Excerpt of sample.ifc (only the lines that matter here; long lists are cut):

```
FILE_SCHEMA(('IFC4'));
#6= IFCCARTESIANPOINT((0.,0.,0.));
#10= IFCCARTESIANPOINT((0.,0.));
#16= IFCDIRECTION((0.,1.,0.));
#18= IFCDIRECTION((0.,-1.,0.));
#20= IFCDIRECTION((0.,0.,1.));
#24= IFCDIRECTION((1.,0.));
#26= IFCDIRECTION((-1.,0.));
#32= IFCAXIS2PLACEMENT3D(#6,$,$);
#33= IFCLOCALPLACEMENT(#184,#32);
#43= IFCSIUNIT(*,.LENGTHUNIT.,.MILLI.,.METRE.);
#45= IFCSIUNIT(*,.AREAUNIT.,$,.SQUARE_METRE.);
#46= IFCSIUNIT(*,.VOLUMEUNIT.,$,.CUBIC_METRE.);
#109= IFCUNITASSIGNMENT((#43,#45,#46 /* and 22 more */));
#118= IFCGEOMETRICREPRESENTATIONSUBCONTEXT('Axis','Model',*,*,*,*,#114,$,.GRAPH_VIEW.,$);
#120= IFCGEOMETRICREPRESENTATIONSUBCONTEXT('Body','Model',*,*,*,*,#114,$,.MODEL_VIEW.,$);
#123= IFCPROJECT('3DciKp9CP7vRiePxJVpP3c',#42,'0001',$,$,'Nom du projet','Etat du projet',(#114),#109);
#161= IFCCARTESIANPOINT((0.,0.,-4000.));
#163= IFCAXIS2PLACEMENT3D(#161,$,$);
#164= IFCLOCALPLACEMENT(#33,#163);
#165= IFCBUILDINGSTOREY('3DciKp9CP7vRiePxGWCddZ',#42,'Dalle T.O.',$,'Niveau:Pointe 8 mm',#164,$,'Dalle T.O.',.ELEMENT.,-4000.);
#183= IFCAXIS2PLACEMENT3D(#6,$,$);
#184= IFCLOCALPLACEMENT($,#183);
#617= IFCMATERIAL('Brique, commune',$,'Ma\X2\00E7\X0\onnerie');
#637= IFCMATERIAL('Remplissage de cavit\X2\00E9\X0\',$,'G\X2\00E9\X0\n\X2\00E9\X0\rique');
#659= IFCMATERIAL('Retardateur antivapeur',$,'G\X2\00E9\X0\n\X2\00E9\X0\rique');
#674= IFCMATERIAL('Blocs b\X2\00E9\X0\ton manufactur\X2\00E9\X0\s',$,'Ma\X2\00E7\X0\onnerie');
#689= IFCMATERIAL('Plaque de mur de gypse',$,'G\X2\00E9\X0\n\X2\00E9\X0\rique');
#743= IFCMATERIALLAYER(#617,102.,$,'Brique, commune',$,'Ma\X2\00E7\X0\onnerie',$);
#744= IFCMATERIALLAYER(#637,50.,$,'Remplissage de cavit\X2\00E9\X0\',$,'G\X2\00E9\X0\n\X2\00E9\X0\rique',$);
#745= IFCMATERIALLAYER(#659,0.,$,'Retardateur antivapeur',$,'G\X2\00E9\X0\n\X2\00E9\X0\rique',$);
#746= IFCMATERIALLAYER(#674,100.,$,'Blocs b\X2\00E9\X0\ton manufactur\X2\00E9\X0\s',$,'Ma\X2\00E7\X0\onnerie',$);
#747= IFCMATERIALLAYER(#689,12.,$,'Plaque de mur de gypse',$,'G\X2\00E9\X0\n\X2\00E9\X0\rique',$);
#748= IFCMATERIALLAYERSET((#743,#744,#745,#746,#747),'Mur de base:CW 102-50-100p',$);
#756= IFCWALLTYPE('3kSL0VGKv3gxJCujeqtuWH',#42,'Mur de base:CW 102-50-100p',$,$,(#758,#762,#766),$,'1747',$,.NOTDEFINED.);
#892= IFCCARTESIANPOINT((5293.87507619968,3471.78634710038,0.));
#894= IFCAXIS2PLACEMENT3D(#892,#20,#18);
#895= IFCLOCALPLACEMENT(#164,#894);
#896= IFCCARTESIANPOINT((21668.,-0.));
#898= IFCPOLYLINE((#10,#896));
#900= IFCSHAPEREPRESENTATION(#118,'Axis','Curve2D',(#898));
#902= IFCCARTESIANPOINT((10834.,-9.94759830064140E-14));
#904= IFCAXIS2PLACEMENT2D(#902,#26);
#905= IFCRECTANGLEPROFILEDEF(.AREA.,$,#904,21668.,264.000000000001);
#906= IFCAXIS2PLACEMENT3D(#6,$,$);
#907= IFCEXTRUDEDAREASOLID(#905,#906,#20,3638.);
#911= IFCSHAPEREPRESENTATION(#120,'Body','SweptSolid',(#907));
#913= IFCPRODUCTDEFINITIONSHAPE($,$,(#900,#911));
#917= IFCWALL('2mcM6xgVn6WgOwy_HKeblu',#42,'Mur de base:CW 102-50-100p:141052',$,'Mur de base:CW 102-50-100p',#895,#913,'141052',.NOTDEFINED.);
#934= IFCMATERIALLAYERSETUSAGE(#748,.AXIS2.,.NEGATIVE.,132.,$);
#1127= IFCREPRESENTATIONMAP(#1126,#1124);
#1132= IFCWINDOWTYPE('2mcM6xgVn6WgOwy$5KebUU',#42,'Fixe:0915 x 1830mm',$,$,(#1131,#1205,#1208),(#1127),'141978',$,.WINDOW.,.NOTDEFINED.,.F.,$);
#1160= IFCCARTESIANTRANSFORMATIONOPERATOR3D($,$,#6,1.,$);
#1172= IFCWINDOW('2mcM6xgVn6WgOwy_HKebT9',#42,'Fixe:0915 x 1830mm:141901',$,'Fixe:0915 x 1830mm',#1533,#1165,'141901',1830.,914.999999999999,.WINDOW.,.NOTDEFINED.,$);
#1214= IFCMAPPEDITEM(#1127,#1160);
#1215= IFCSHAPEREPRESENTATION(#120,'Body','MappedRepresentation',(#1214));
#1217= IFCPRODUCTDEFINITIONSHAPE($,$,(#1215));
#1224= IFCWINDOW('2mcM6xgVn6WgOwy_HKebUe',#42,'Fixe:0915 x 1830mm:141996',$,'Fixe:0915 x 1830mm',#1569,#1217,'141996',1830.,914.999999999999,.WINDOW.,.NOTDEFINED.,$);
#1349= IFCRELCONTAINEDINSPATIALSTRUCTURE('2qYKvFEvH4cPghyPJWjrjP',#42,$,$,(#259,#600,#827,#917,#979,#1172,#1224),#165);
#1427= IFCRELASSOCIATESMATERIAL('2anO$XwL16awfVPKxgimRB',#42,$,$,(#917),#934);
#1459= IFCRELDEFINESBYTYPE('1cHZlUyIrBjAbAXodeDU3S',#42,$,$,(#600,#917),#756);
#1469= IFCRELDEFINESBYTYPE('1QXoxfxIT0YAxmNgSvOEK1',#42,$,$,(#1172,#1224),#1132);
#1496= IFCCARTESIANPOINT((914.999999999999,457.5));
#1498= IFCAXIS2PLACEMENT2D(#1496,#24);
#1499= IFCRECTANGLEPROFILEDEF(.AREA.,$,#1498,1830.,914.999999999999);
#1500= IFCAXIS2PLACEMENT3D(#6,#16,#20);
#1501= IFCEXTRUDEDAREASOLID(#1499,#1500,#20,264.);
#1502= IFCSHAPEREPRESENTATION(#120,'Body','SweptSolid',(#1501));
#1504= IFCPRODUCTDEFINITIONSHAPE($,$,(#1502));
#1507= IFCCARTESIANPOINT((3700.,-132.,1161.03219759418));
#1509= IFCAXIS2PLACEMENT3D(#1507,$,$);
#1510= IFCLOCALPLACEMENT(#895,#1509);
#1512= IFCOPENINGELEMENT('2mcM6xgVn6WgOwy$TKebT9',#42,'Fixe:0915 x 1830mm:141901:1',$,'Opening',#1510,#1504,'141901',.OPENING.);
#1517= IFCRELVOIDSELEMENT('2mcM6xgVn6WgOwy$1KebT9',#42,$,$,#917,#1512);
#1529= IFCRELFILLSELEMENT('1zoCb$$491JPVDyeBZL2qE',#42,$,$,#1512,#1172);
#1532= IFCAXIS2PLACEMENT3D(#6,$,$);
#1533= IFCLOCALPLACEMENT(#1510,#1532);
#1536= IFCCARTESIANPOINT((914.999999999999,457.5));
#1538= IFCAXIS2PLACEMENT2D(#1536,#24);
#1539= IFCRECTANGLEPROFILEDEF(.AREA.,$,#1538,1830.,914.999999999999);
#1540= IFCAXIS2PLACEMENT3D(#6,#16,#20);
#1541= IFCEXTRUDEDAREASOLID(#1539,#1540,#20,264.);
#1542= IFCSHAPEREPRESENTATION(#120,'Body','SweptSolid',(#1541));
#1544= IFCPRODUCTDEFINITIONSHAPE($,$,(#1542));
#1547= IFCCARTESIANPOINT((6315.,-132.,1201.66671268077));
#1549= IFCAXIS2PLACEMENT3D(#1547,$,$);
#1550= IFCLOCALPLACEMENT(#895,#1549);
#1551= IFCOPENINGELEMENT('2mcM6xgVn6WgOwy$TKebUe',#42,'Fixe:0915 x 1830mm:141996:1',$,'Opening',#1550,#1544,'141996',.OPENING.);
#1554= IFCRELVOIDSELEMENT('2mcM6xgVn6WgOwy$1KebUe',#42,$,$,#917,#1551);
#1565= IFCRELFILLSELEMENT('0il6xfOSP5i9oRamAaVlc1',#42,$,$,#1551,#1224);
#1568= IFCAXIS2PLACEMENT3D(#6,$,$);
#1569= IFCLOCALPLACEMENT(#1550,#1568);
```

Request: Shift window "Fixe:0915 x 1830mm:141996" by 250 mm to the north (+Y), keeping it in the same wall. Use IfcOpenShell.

```python
import ifcopenshell
import ifcopenshell.api.geometry
import ifcopenshell.util.placement
import ifcopenshell.util.unit

model = ifcopenshell.open("sample.ifc")
unit_scale = ifcopenshell.util.unit.calculate_unit_scale(model)

window = model.by_guid("2mcM6xgVn6WgOwy_HKebUe")
opening = window.FillsVoids[0].RelatingOpeningElement
wall = opening.VoidsElements[0].RelatingBuildingElement

wall_matrix = ifcopenshell.util.placement.get_local_placement(wall.ObjectPlacement)
shift = wall_matrix[:3, 0] * -0.25 / unit_scale
before = ifcopenshell.util.placement.get_local_placement(window.ObjectPlacement)[:3, 3].copy()

# The window is placed relative to its opening, so it follows when the opening moves.
matrix = ifcopenshell.util.placement.get_local_placement(opening.ObjectPlacement)
matrix[:3, 3] += shift
ifcopenshell.api.geometry.edit_object_placement(
    model, product=opening, matrix=matrix, is_si=False, should_transform_children=True
)

after = ifcopenshell.util.placement.get_local_placement(window.ObjectPlacement)[:3, 3]
print("window moved by", (after - before).round(3) + 0.0)

model.write("sample_edited.ifc")
```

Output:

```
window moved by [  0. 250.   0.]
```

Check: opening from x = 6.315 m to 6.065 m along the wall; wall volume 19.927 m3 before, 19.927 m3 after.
